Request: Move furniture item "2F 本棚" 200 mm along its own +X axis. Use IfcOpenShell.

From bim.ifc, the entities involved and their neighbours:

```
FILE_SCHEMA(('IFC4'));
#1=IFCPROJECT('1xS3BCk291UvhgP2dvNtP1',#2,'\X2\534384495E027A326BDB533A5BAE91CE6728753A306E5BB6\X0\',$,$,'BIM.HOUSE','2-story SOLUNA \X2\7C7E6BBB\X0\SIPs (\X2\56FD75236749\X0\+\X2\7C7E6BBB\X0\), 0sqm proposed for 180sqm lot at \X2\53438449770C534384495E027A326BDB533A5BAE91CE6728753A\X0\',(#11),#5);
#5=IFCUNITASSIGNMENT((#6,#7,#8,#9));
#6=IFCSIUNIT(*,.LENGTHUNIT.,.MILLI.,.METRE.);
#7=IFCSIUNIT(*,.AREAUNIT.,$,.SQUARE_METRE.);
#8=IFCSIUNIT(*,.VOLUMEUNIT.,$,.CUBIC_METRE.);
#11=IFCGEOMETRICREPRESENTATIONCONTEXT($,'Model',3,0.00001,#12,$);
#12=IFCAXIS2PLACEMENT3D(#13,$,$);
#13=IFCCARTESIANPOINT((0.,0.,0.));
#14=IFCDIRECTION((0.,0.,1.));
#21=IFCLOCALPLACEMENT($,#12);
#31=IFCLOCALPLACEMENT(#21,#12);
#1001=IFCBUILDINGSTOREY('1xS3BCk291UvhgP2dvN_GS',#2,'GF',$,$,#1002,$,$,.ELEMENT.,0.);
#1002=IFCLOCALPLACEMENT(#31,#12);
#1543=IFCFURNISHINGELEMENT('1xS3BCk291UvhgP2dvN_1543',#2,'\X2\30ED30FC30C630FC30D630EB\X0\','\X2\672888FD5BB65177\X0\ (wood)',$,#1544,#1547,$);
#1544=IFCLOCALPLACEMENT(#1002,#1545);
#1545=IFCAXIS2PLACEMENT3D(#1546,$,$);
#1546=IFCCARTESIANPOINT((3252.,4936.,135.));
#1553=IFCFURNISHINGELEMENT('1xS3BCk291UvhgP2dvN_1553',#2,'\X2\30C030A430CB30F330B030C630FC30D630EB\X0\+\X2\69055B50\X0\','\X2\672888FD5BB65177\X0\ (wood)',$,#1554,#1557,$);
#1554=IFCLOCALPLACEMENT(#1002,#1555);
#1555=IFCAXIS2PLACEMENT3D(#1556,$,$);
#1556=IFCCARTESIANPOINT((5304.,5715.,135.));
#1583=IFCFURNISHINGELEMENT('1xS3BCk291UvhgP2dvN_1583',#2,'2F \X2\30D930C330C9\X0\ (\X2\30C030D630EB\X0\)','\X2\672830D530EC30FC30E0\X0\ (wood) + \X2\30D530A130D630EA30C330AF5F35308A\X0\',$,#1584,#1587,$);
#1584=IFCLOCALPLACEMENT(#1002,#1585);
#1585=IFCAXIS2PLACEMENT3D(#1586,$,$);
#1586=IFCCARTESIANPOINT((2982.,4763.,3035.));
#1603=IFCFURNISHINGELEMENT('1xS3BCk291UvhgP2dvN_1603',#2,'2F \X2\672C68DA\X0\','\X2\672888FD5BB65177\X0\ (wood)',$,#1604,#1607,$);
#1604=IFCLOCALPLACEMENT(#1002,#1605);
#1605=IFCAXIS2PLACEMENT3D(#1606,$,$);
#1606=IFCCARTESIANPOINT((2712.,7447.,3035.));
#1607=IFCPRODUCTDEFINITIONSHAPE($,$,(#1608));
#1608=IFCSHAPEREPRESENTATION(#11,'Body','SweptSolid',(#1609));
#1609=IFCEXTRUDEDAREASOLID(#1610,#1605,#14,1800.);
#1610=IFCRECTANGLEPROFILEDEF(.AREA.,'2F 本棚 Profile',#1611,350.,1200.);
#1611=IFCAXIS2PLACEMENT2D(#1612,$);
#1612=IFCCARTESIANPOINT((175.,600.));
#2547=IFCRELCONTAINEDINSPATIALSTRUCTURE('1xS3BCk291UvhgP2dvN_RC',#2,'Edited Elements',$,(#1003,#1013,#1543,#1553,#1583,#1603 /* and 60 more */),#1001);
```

```python
import ifcopenshell
import ifcopenshell.api.geometry
import ifcopenshell.util.placement
import ifcopenshell.util.unit

model = ifcopenshell.open("bim.ifc")
unit_scale = ifcopenshell.util.unit.calculate_unit_scale(model)

item = model.by_guid("1xS3BCk291UvhgP2dvN_1603")
matrix = ifcopenshell.util.placement.get_local_placement(item.ObjectPlacement)
matrix[:3, 3] += matrix[:3, 0] * 0.2 / unit_scale
ifcopenshell.api.geometry.edit_object_placement(model, product=item, matrix=matrix, is_si=False)

print(ifcopenshell.util.placement.get_local_placement(item.ObjectPlacement).round(3) + 0.0)

model.write("bim_updated.ifc")
```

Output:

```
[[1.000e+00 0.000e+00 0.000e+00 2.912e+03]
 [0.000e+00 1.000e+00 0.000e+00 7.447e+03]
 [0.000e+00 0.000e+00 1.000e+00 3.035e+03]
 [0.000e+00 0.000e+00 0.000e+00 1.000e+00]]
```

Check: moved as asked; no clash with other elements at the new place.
